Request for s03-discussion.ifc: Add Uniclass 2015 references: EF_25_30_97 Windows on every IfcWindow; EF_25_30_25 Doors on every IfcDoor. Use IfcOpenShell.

First a look at what the model holds.

```python
import ifcopenshell

model = ifcopenshell.open("s03-discussion.ifc")
print(model.schema)
print("classifications:", [c.Name for c in model.by_type("IfcClassification")])
for ifc_class in ("IfcDoor", "IfcRoof", "IfcStair", "IfcWall", "IfcWindow"):
    print(ifc_class, len(model.by_type(ifc_class)))
```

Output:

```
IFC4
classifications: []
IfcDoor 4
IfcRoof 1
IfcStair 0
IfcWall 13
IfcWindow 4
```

```python
import ifcopenshell
import ifcopenshell.api.classification

model = ifcopenshell.open("s03-discussion.ifc")

system = ifcopenshell.api.classification.add_classification(model, classification="Uniclass 2015")

codes = {
    "IfcWindow": ("EF_25_30_97", "Windows"),
    "IfcDoor": ("EF_25_30_25", "Doors"),
}
for ifc_class, (code, name) in codes.items():
    products = model.by_type(ifc_class)
    ifcopenshell.api.classification.add_reference(
        model, products=products, classification=system, identification=code, name=name
    )
    print(code, len(products))

model.write("s03-discussion-out.ifc")
```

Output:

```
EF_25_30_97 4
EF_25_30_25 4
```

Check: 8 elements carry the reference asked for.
